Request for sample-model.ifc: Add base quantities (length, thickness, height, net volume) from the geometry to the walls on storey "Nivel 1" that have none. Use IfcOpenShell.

First a look at what the model holds.

```python
import ifcopenshell
import ifcopenshell.util.element
import ifcopenshell.util.unit

model = ifcopenshell.open("sample-model.ifc")
print(model.schema)
for unit_type in ("LENGTHUNIT", "AREAUNIT", "VOLUMEUNIT"):
    print(unit_type, ifcopenshell.util.unit.calculate_unit_scale(model, unit_type))
storey = next(s for s in model.by_type("IfcBuildingStorey") if s.Name == "Nivel 1")
walls = [e for e in ifcopenshell.util.element.get_decomposition(storey) if e.is_a("IfcWall")]
for e in sorted(walls, key=lambda e: e.id()):
    print(e.id(), e.is_a(), e.Name, list(ifcopenshell.util.element.get_psets(e, qtos_only=True)), sep=" | ")
```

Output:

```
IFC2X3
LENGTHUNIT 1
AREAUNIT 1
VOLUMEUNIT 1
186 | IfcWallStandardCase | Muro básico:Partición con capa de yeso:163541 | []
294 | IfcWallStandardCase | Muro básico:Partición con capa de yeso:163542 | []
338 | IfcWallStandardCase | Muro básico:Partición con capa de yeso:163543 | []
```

```python
import ifcopenshell
import ifcopenshell.api.pset
import ifcopenshell.geom
import ifcopenshell.util.element
import ifcopenshell.util.shape
import ifcopenshell.util.unit

model = ifcopenshell.open("sample-model.ifc")
unit_scale = ifcopenshell.util.unit.calculate_unit_scale(model)
volume_scale = ifcopenshell.util.unit.calculate_unit_scale(model, "VOLUMEUNIT")
settings = ifcopenshell.geom.settings()

storey = next(s for s in model.by_type("IfcBuildingStorey") if s.Name == "Nivel 1")
walls = [e for e in ifcopenshell.util.element.get_decomposition(storey) if e.is_a("IfcWall")]

for e in sorted(walls, key=lambda e: e.id()):
    if ifcopenshell.util.element.get_psets(e, qtos_only=True, should_inherit=False):
        continue
    # Geometry comes back in metres, in the element's own axes.
    shape = ifcopenshell.geom.create_shape(settings, e)
    values = {
        "Length": ifcopenshell.util.shape.get_x(shape.geometry) / unit_scale,
        "Width": ifcopenshell.util.shape.get_y(shape.geometry) / unit_scale,
        "Height": ifcopenshell.util.shape.get_z(shape.geometry) / unit_scale,
        "NetVolume": ifcopenshell.util.shape.get_volume(shape.geometry) / volume_scale,
    }
    qto = ifcopenshell.api.pset.add_qto(model, product=e, name="BaseQuantities")
    ifcopenshell.api.pset.edit_qto(model, qto=qto, properties=values)
    print(e.id(), {k: round(v, 3) for k, v in values.items()})

model.write("sample-model_edited.ifc")
```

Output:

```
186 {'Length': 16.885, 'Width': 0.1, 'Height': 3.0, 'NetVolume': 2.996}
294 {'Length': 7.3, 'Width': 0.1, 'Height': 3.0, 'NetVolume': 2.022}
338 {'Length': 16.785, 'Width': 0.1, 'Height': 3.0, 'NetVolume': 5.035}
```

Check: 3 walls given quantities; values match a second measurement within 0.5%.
